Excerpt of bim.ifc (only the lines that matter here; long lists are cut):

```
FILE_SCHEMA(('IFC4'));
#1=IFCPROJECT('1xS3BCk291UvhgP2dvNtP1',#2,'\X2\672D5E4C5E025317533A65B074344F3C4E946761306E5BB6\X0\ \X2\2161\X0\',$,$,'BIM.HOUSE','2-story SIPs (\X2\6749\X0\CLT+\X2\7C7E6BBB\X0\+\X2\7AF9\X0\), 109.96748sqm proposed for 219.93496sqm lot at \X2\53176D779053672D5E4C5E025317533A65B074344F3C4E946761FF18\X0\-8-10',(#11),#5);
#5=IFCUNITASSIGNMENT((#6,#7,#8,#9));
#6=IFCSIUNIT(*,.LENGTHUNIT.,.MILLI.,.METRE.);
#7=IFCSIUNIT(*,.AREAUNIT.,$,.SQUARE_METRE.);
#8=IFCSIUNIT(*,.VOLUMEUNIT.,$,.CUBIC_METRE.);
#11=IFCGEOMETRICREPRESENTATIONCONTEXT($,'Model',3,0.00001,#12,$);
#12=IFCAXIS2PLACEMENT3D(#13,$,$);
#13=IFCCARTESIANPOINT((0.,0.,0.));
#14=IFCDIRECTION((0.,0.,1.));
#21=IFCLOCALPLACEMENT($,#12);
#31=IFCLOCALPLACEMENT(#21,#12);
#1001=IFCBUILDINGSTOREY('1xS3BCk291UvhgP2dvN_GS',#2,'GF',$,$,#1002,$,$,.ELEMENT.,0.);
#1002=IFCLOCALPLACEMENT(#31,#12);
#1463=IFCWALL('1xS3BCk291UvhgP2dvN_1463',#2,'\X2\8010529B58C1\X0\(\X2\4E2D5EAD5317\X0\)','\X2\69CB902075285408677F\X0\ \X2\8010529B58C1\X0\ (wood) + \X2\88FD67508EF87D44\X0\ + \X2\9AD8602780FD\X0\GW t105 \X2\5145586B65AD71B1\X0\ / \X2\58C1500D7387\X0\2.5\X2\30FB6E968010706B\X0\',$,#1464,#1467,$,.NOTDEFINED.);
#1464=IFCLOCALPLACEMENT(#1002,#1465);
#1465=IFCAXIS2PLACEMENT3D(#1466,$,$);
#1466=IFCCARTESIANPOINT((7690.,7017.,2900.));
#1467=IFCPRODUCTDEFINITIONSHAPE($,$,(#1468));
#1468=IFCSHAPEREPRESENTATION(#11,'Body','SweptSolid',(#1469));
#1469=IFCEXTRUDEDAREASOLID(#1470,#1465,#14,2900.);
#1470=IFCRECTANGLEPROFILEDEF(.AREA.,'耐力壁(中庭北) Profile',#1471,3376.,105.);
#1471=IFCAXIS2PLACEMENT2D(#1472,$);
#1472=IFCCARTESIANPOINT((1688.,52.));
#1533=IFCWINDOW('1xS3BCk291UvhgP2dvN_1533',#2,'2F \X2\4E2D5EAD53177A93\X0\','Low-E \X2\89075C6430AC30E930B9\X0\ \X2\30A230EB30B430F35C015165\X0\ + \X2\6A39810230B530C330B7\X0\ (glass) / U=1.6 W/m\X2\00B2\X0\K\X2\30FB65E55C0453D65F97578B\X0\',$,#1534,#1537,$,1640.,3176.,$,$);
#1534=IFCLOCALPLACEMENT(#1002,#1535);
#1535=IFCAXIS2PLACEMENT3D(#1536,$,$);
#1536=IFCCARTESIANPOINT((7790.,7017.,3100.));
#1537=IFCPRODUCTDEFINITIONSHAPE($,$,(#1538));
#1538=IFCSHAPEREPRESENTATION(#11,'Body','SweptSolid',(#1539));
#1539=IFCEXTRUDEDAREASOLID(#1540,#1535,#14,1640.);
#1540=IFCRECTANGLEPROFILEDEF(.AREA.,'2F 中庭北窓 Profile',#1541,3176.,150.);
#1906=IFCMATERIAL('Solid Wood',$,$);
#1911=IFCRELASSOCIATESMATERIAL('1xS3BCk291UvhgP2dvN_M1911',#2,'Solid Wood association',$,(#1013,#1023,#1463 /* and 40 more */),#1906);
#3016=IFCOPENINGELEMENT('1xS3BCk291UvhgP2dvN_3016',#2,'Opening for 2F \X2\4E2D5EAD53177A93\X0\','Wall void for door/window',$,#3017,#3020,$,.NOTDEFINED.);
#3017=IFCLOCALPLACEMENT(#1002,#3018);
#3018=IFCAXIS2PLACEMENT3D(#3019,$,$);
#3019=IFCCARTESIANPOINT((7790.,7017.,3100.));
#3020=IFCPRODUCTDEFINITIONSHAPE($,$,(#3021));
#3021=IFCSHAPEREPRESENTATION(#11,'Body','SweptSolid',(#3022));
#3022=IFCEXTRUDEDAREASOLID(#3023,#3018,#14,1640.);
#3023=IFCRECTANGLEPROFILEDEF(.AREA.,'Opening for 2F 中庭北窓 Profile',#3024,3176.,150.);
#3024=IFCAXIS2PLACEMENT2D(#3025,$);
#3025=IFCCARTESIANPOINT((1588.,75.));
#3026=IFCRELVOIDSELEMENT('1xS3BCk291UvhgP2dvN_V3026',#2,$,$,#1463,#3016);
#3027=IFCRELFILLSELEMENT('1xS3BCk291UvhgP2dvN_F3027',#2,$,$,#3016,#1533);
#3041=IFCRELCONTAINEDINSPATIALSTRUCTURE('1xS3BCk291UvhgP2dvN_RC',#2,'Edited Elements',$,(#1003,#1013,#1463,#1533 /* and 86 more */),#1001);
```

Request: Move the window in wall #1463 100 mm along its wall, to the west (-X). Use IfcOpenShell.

```python
import ifcopenshell
import ifcopenshell.api.geometry
import ifcopenshell.util.placement

model = ifcopenshell.open("bim.ifc")

window = model.by_guid("1xS3BCk291UvhgP2dvN_1533")
opening = window.FillsVoids[0].RelatingOpeningElement
wall = opening.VoidsElements[0].RelatingBuildingElement

wall_matrix = ifcopenshell.util.placement.get_local_placement(wall.ObjectPlacement)
shift = wall_matrix[:3, 0] * -100.0
before = ifcopenshell.util.placement.get_local_placement(window.ObjectPlacement)[:3, 3].copy()

# The window is not placed relative to its opening, so move both.
for product in (opening, window):
    matrix = ifcopenshell.util.placement.get_local_placement(product.ObjectPlacement)
    matrix[:3, 3] += shift
    ifcopenshell.api.geometry.edit_object_placement(model, product=product, matrix=matrix, is_si=False)

after = ifcopenshell.util.placement.get_local_placement(window.ObjectPlacement)[:3, 3]
print("window moved by", (after - before).round(3) + 0.0)

model.write("bim_v2.ifc")
```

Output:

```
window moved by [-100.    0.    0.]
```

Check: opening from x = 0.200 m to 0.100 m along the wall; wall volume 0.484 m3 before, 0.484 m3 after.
